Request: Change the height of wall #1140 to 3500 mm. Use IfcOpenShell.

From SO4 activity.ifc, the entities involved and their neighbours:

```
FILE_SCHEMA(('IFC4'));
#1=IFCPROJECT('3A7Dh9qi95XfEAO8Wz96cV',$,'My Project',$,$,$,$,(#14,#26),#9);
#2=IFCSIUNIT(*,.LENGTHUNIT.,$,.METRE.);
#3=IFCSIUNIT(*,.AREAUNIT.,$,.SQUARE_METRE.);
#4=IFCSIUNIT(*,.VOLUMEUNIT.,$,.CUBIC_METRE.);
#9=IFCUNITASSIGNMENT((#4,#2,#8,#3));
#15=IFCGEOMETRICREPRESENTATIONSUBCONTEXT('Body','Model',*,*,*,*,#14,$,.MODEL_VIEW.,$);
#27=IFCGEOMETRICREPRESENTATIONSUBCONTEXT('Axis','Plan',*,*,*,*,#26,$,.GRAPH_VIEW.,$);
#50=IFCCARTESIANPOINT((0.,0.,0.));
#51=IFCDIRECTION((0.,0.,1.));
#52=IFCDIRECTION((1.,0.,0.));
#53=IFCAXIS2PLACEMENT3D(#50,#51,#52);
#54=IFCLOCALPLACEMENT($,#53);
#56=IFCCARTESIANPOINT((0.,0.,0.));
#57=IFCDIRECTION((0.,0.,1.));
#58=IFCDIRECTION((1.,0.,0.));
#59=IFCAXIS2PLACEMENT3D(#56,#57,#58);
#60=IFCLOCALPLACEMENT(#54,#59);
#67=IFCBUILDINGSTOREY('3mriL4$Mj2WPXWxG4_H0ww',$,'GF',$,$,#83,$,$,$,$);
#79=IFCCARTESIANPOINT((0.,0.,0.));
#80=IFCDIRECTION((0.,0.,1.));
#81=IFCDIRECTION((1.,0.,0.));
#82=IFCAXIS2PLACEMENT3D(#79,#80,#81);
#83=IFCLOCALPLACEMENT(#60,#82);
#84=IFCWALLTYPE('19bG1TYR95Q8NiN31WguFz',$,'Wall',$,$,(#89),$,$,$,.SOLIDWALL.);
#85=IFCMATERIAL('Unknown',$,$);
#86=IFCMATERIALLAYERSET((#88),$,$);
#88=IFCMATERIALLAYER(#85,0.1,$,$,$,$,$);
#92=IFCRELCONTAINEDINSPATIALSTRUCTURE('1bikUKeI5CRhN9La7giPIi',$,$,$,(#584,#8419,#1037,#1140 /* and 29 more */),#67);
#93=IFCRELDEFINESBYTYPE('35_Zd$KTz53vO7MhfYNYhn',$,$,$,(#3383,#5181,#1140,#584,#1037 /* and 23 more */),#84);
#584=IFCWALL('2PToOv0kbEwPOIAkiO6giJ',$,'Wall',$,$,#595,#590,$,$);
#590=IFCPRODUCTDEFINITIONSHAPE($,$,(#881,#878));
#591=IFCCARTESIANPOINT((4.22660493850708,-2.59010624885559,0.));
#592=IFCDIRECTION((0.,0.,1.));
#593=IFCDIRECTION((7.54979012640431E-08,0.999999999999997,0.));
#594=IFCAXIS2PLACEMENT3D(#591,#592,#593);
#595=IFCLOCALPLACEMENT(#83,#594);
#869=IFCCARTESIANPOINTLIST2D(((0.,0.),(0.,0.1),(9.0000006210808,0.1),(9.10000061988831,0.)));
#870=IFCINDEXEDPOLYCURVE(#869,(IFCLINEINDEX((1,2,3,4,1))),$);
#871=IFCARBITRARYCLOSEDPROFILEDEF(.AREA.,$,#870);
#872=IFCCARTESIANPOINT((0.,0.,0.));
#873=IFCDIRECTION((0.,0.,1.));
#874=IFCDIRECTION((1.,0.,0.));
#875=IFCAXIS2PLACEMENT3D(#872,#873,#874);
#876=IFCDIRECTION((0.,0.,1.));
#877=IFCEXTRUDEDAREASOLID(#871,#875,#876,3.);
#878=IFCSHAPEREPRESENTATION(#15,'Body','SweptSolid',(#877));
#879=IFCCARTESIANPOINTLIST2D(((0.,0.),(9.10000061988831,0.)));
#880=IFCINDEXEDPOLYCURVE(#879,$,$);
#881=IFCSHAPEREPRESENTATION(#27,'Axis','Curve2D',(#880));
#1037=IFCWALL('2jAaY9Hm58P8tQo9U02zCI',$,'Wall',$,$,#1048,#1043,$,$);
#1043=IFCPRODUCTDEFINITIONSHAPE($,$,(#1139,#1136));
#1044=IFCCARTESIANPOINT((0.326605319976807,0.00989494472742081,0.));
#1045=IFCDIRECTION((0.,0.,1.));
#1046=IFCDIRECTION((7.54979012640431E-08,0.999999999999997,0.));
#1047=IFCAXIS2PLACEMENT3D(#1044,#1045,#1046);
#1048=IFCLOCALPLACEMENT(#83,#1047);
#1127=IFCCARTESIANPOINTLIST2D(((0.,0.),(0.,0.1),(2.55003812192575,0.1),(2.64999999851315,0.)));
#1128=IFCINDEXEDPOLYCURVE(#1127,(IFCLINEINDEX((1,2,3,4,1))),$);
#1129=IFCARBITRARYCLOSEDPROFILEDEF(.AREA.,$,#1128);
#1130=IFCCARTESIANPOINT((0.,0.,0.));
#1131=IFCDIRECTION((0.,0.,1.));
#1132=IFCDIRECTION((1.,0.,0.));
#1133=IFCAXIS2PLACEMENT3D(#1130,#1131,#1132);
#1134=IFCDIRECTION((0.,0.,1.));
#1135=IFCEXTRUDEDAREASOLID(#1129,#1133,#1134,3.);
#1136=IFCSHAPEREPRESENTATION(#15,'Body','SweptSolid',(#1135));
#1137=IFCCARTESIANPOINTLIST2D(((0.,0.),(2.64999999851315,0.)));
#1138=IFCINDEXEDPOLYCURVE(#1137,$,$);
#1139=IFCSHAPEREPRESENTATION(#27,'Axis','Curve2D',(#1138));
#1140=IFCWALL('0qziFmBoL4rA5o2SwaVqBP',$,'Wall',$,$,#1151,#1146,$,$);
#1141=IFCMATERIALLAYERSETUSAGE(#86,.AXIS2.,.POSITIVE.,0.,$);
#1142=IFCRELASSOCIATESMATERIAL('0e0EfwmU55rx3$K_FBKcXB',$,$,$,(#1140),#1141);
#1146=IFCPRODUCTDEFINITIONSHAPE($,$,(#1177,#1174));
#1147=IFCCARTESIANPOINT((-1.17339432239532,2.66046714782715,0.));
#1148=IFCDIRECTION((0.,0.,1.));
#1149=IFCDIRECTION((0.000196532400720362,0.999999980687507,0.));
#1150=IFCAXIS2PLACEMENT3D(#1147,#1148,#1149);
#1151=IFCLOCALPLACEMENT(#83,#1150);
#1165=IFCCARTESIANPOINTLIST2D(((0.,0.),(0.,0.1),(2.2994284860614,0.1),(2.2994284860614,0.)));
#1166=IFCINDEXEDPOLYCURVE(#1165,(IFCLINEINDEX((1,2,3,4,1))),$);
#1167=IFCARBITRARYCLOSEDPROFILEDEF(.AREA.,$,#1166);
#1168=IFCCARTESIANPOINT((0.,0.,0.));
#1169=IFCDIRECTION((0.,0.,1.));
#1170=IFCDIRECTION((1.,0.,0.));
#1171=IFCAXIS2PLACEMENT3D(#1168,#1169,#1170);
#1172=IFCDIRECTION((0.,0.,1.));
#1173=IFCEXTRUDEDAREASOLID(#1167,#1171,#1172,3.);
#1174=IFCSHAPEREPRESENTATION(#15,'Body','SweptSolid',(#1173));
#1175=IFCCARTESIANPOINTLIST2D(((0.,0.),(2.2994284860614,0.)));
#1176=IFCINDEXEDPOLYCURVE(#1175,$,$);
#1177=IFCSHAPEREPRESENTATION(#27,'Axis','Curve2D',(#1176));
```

```python
import ifcopenshell
import ifcopenshell.geom
import ifcopenshell.util.representation
import ifcopenshell.util.shape

model = ifcopenshell.open("SO4 activity.ifc")
settings = ifcopenshell.geom.settings()


def volume(element):
    """Net volume in cubic metres, openings subtracted."""
    shape = ifcopenshell.geom.create_shape(settings, element)
    return ifcopenshell.util.shape.get_volume(shape.geometry)


wall = model.by_guid("0qziFmBoL4rA5o2SwaVqBP")
before = volume(wall)

body = ifcopenshell.util.representation.get_representation(wall, "Model", "Body")
solid = body.Items[0]
old_height = solid.Depth
solid.Depth = 3.5
after = volume(wall)

print(f"height {old_height:g} -> {solid.Depth:g}, volume {before:.3f} -> {after:.3f} m3")

model.write("SO4 activity_v2.ifc")
```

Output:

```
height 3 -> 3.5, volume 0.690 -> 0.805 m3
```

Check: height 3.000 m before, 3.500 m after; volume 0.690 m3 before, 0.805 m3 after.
